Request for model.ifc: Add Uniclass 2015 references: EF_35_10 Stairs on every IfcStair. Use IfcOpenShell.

First a look at what the model holds.

```python
import ifcopenshell

model = ifcopenshell.open("model.ifc")
print(model.schema)
print("classifications:", [c.Name for c in model.by_type("IfcClassification")])
for ifc_class in ("IfcDoor", "IfcRoof", "IfcStair", "IfcWall", "IfcWindow"):
    print(ifc_class, len(model.by_type(ifc_class)))
```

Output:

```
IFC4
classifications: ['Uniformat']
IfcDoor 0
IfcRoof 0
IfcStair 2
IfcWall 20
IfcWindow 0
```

```python
import ifcopenshell
import ifcopenshell.api.classification

model = ifcopenshell.open("model.ifc")

system = ifcopenshell.api.classification.add_classification(model, classification="Uniclass 2015")

codes = {
    "IfcStair": ("EF_35_10", "Stairs"),
}
for ifc_class, (code, name) in codes.items():
    products = model.by_type(ifc_class)
    ifcopenshell.api.classification.add_reference(
        model, products=products, classification=system, identification=code, name=name
    )
    print(code, len(products))

model.write("model_edited.ifc")
```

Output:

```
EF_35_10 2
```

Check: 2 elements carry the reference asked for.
